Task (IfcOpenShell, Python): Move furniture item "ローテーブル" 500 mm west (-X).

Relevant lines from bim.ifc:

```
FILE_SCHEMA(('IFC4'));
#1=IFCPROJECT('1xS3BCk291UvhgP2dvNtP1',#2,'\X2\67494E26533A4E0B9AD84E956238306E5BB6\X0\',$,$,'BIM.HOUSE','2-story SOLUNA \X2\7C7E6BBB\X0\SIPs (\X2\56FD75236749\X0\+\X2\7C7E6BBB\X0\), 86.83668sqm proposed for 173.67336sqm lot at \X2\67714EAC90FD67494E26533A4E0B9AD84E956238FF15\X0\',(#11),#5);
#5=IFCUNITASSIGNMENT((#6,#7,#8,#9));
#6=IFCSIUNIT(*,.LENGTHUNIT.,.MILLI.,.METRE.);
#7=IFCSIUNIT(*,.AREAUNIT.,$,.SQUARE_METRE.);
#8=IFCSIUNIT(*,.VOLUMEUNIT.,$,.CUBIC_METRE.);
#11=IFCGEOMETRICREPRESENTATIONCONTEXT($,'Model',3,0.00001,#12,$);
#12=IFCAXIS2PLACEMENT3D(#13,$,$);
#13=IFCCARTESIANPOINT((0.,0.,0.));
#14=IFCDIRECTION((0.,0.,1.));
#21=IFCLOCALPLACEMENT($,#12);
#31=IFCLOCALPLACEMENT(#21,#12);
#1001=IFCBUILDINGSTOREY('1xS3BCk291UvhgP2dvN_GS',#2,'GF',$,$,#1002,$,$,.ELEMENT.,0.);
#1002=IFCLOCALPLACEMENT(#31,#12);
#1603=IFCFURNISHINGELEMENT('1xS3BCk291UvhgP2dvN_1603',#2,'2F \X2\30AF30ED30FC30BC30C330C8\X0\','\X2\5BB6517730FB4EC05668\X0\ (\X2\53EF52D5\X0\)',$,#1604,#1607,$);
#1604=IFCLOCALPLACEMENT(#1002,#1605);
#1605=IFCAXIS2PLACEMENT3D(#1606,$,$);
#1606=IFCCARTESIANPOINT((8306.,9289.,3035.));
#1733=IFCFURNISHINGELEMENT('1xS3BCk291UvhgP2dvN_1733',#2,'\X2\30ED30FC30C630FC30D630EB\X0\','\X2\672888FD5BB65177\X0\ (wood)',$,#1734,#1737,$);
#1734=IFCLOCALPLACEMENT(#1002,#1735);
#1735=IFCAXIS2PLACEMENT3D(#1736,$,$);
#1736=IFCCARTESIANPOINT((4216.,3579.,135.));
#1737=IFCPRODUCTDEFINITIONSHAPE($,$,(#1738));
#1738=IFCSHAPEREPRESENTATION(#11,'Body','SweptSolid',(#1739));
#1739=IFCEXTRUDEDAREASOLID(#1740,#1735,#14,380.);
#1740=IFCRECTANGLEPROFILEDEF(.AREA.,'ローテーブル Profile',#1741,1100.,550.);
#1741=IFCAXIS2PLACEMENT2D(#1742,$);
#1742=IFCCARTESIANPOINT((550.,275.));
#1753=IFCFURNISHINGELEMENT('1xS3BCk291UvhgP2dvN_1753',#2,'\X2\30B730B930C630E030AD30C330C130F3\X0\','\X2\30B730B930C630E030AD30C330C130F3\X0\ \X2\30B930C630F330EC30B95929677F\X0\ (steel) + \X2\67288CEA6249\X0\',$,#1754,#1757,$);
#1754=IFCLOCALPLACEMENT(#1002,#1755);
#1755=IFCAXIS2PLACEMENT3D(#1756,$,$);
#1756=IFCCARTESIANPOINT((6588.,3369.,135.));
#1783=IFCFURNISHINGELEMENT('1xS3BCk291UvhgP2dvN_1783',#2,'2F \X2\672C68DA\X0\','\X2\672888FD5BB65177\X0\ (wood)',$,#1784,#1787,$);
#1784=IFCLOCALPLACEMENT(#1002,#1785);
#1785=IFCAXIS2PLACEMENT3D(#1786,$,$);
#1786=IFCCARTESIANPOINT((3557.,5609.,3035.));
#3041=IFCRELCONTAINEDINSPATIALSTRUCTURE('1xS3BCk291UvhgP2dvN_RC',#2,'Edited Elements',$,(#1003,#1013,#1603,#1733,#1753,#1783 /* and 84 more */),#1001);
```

```python
import ifcopenshell
import ifcopenshell.api.geometry
import ifcopenshell.util.placement

model = ifcopenshell.open("bim.ifc")

item = model.by_guid("1xS3BCk291UvhgP2dvN_1733")
matrix = ifcopenshell.util.placement.get_local_placement(item.ObjectPlacement)
matrix[0, 3] -= 500.0
ifcopenshell.api.geometry.edit_object_placement(model, product=item, matrix=matrix, is_si=False)

print(ifcopenshell.util.placement.get_local_placement(item.ObjectPlacement).round(3) + 0.0)

model.write("bim_edited.ifc")
```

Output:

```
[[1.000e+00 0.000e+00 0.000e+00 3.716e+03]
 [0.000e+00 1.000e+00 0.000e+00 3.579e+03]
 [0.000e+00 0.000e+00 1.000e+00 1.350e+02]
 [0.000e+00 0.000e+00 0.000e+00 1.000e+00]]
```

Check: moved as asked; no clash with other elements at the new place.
